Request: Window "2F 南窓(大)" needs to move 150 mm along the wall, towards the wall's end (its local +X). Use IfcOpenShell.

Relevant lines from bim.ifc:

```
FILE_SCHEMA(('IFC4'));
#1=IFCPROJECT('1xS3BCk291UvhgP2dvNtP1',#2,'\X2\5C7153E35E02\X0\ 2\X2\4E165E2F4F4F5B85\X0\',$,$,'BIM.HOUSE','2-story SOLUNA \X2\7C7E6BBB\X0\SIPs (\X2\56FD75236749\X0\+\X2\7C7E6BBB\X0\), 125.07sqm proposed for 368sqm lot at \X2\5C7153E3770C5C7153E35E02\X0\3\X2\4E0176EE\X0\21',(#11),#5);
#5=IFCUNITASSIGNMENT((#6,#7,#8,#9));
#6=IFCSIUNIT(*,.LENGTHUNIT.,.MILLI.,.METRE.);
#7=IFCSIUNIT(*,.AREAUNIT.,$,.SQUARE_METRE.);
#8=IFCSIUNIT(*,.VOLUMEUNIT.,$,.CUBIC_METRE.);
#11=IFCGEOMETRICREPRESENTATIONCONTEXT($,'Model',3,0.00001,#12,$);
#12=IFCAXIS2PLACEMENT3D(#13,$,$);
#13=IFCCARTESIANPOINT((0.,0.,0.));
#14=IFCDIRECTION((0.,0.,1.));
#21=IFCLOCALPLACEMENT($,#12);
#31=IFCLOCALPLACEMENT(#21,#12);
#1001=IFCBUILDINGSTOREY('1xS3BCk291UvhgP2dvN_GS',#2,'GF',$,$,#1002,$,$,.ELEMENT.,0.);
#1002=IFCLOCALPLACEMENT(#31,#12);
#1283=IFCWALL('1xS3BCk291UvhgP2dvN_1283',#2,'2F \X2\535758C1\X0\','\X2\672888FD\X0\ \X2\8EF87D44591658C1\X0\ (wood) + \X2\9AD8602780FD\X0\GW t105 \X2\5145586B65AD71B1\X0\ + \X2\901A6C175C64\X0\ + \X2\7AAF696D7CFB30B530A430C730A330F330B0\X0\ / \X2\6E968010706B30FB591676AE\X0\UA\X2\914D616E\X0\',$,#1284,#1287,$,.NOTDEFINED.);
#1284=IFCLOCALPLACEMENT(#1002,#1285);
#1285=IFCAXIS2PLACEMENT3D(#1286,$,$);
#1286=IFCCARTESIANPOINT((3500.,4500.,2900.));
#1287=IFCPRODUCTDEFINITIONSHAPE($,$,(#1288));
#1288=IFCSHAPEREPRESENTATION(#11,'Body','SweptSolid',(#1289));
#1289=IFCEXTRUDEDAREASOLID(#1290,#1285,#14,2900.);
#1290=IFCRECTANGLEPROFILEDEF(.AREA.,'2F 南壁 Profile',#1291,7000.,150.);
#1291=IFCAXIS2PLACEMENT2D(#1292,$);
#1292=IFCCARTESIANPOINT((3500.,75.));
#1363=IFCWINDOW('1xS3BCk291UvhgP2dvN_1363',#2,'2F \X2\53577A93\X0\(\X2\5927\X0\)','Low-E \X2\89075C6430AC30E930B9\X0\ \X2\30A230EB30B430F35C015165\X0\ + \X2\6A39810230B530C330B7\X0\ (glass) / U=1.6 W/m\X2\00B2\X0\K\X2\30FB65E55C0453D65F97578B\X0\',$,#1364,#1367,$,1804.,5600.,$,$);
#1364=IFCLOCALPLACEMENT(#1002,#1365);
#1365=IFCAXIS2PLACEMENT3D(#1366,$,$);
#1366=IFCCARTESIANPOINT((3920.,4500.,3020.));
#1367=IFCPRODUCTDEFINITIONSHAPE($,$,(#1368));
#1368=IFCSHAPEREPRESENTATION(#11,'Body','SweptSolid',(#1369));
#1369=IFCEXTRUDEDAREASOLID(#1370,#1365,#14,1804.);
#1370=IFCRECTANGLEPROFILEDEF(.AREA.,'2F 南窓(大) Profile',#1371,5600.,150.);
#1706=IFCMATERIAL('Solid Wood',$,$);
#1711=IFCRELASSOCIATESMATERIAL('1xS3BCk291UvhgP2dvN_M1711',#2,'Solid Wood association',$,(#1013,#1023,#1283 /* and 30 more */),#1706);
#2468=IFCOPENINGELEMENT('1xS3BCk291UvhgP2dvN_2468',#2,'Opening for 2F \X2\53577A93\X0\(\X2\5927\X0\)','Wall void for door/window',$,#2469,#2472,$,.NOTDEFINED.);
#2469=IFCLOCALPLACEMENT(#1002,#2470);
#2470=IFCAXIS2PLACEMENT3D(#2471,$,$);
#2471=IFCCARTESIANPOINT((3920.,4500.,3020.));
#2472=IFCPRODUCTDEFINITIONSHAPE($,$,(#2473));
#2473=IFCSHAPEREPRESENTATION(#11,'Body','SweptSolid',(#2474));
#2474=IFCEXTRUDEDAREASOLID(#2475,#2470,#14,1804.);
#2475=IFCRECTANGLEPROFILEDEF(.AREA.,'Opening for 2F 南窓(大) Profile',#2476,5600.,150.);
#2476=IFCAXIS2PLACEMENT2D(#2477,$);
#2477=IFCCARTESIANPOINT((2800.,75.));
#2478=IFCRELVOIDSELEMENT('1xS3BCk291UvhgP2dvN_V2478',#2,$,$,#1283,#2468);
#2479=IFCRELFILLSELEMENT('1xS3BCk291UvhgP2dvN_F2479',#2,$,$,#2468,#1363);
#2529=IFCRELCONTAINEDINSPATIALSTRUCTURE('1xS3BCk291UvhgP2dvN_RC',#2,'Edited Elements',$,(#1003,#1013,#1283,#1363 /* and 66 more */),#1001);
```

```python
import ifcopenshell
import ifcopenshell.api.geometry
import ifcopenshell.util.placement
import ifcopenshell.util.unit

model = ifcopenshell.open("bim.ifc")
unit_scale = ifcopenshell.util.unit.calculate_unit_scale(model)

window = model.by_guid("1xS3BCk291UvhgP2dvN_1363")
opening = window.FillsVoids[0].RelatingOpeningElement
wall = opening.VoidsElements[0].RelatingBuildingElement

wall_matrix = ifcopenshell.util.placement.get_local_placement(wall.ObjectPlacement)
shift = wall_matrix[:3, 0] * 0.15 / unit_scale
before = ifcopenshell.util.placement.get_local_placement(window.ObjectPlacement)[:3, 3].copy()

# The window is not placed relative to its opening, so move both.
for product in (opening, window):
    matrix = ifcopenshell.util.placement.get_local_placement(product.ObjectPlacement)
    matrix[:3, 3] += shift
    ifcopenshell.api.geometry.edit_object_placement(model, product=product, matrix=matrix, is_si=False)

after = ifcopenshell.util.placement.get_local_placement(window.ObjectPlacement)[:3, 3]
print("window moved by", (after - before).round(3) + 0.0)

model.write("bim_rev.ifc")
```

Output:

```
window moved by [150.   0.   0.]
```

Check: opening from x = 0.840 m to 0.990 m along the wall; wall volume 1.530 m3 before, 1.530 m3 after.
